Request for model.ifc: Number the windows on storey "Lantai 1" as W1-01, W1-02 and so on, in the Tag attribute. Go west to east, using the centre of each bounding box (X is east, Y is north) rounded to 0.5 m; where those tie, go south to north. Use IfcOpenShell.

First a look at what the model holds.

```python
import ifcopenshell
import ifcopenshell.util.element
import ifcopenshell.util.placement

model = ifcopenshell.open("model.ifc")
print(model.schema)
storey = next(s for s in model.by_type("IfcBuildingStorey") if s.Name == "Lantai 1")
windows = [e for e in ifcopenshell.util.element.get_decomposition(storey) if e.is_a("IfcWindow")]
for e in sorted(windows, key=lambda e: e.id()):
    origin = ifcopenshell.util.placement.get_local_placement(e.ObjectPlacement)[:3, 3]
    print(e.id(), e.Tag, e.Name, origin.round(2) + 0.0, sep=" | ")
```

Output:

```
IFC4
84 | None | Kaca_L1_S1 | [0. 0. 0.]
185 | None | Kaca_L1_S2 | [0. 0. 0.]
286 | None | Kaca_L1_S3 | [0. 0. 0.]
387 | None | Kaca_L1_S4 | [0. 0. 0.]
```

```python
import ifcopenshell
import ifcopenshell.geom
import ifcopenshell.util.element
import ifcopenshell.util.shape

model = ifcopenshell.open("model.ifc")
settings = ifcopenshell.geom.settings()
settings.set("use-world-coords", True)


def centre(element):
    shape = ifcopenshell.geom.create_shape(settings, element)
    return ifcopenshell.util.shape.get_bbox_centroid(shape.geometry)


storey = next(s for s in model.by_type("IfcBuildingStorey") if s.Name == "Lantai 1")
windows = [e for e in ifcopenshell.util.element.get_decomposition(storey) if e.is_a("IfcWindow")]

# Insertion points can sit at a corner or the storey origin, so sort by the geometry (in metres).
centres = {e: centre(e) for e in windows}
windows.sort(key=lambda e: (round(centres[e][0] / 0.5), centres[e][1]))

for i, e in enumerate(windows, start=1):
    number = f"W1-{i:02d}"
    e.Tag = number
    print(e.id(), number)

model.write("model_edited.ifc")
```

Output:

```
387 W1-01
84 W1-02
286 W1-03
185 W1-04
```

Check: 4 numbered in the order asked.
